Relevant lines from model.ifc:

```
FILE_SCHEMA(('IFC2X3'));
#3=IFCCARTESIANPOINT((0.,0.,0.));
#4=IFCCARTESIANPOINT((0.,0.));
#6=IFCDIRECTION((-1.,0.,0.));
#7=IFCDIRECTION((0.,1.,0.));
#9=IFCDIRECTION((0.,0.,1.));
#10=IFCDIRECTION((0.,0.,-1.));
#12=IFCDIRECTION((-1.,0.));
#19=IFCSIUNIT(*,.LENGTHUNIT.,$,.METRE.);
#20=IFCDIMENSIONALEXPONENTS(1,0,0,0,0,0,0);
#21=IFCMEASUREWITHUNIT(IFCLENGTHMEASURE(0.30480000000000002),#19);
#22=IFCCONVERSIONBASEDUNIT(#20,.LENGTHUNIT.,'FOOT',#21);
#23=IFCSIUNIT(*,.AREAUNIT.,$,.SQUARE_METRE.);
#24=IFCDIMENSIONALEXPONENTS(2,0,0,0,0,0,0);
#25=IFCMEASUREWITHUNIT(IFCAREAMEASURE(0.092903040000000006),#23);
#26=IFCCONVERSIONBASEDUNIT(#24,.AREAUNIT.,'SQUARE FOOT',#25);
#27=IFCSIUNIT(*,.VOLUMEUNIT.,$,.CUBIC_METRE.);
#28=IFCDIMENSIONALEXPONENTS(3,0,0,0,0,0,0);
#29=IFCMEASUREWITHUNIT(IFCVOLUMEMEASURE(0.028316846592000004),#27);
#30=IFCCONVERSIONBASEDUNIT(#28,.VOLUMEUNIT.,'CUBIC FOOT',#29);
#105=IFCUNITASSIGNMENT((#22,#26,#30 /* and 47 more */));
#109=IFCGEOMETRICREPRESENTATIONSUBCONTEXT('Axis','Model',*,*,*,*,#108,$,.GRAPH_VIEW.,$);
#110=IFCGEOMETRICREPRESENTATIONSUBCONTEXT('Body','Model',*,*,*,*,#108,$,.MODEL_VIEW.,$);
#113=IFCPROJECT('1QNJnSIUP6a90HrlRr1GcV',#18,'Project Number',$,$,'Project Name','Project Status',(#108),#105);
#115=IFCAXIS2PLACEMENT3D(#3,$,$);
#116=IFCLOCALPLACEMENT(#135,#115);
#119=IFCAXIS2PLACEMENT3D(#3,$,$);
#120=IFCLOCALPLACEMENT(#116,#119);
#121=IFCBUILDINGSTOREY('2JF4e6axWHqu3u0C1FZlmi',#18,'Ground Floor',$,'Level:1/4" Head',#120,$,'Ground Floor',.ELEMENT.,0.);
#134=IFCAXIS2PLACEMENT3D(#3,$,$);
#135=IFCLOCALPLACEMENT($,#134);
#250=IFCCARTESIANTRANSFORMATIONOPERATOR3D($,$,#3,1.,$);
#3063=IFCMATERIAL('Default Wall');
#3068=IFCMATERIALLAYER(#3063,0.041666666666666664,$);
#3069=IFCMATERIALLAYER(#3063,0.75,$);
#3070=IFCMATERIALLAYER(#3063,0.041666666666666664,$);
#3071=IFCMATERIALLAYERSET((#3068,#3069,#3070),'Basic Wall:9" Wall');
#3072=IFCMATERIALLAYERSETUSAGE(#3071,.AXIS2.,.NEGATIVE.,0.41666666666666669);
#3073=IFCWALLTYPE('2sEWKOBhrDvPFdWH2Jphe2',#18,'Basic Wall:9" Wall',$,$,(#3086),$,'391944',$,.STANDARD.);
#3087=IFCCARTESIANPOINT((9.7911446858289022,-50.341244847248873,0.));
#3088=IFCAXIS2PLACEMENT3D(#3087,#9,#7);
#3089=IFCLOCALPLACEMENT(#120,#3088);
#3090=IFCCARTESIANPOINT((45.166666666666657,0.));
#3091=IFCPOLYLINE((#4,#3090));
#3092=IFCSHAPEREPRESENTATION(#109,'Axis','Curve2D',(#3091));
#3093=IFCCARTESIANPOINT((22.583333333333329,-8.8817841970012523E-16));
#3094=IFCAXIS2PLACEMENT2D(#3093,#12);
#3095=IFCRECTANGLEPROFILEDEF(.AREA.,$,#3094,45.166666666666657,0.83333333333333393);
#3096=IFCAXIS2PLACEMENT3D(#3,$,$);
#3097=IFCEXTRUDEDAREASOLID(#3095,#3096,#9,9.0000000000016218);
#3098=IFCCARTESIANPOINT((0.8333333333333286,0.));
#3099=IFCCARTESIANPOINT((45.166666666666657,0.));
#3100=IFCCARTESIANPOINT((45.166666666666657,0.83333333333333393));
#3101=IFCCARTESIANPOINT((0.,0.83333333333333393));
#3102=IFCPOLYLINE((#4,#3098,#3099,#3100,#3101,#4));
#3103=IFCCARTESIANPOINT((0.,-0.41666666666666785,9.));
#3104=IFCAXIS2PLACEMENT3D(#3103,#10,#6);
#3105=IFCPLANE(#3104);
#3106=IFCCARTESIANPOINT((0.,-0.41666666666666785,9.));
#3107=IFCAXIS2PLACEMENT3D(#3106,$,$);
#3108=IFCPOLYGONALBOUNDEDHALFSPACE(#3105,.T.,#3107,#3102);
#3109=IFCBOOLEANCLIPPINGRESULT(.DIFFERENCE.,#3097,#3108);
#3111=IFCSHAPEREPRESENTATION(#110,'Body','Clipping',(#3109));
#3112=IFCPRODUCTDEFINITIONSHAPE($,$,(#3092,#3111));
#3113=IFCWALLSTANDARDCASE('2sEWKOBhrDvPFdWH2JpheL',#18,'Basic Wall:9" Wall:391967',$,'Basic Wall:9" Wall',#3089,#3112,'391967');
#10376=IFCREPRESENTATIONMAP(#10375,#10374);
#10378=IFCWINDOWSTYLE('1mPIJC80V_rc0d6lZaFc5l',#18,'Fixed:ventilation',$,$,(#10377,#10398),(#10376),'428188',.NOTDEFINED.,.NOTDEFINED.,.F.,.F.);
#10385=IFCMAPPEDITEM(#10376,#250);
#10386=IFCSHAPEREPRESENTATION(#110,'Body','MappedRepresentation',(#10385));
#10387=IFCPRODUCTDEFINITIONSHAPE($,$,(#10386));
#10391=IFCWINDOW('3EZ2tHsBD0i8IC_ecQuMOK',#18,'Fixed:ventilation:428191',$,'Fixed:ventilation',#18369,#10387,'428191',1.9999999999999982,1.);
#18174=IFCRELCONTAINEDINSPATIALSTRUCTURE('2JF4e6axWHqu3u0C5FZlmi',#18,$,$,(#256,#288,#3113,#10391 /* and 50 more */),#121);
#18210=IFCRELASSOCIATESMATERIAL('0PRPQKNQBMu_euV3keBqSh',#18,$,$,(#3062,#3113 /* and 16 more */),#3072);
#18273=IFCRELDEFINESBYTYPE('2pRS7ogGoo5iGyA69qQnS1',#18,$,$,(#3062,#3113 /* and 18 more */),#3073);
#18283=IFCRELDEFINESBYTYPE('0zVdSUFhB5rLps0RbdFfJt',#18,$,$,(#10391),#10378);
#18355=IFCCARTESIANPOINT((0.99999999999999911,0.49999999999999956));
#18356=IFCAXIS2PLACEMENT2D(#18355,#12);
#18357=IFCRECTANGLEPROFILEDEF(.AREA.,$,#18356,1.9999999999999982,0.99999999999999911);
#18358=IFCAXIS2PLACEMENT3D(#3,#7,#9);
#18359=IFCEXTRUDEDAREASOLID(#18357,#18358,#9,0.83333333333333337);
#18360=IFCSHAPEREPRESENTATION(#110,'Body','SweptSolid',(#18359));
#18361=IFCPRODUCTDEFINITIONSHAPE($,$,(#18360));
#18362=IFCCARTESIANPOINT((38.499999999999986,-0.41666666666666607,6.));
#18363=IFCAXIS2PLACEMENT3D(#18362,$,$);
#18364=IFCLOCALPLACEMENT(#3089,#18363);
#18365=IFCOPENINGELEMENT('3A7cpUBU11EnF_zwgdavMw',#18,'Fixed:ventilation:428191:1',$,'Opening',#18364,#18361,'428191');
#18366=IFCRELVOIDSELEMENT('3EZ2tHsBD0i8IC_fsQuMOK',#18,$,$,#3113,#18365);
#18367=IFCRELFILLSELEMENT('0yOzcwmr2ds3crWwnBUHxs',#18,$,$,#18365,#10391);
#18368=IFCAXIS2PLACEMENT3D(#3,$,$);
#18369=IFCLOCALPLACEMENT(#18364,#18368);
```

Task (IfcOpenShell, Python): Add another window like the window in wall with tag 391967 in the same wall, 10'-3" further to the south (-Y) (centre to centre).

```python
import ifcopenshell
import ifcopenshell.api.feature
import ifcopenshell.api.geometry
import ifcopenshell.api.root
import ifcopenshell.geom
import ifcopenshell.util.element
import ifcopenshell.util.placement
import ifcopenshell.util.shape
import ifcopenshell.util.unit

model = ifcopenshell.open("model.ifc")
unit_scale = ifcopenshell.util.unit.calculate_unit_scale(model)
settings = ifcopenshell.geom.settings()


def volume(element):
    """Net volume in cubic metres, openings subtracted."""
    shape = ifcopenshell.geom.create_shape(settings, element)
    return ifcopenshell.util.shape.get_volume(shape.geometry)


def reuse_history(source, copy):
    """copy_class also copies each property set's owner history, people and application; keep the originals."""
    for rel in copy.IsDefinedBy:
        if rel.is_a("IfcRelDefinesByProperties") and (history := rel.RelatingPropertyDefinition.OwnerHistory):
            rel.RelatingPropertyDefinition.OwnerHistory = source.OwnerHistory
            ifcopenshell.util.element.remove_deep2(model, history)


window = model.by_id(10391)
opening = window.FillsVoids[0].RelatingOpeningElement
wall = opening.VoidsElements[0].RelatingBuildingElement
before = volume(wall)
shift = ifcopenshell.util.placement.get_local_placement(wall.ObjectPlacement)[:3, 0] * -123 * 0.0254 / unit_scale

# copy_class copies the void relationship, type, container and properties, but no geometry.
new_opening = ifcopenshell.api.root.copy_class(model, product=opening)
new_opening.Representation = ifcopenshell.util.element.copy_deep(
    model, opening.Representation, exclude=["IfcGeometricRepresentationContext", "IfcRepresentationMap"]
)
new_opening.Name = "Fixed:ventilation"
new_opening.Tag = None
new_window = ifcopenshell.api.root.copy_class(model, product=window)
new_window.Representation = ifcopenshell.util.element.copy_deep(
    model, window.Representation, exclude=["IfcGeometricRepresentationContext", "IfcRepresentationMap"]
)
new_window.Name = "Fixed:ventilation"
new_window.Tag = None
reuse_history(window, new_window)
fills = ifcopenshell.api.feature.add_filling(model, opening=new_opening, element=new_window)
fills.OwnerHistory = new_window.OwnerHistory  # required in IFC2X3

for old, new in ((opening, new_opening), (window, new_window)):
    matrix = ifcopenshell.util.placement.get_local_placement(old.ObjectPlacement)
    matrix[:3, 3] += shift
    ifcopenshell.api.geometry.edit_object_placement(model, product=new, matrix=matrix, is_si=False)

after = volume(wall)

print(f"wall volume {before:.3f} -> {after:.3f} m3")

model.write("model_v2.ifc")
```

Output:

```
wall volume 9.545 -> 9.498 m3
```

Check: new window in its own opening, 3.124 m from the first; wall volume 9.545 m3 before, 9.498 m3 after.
